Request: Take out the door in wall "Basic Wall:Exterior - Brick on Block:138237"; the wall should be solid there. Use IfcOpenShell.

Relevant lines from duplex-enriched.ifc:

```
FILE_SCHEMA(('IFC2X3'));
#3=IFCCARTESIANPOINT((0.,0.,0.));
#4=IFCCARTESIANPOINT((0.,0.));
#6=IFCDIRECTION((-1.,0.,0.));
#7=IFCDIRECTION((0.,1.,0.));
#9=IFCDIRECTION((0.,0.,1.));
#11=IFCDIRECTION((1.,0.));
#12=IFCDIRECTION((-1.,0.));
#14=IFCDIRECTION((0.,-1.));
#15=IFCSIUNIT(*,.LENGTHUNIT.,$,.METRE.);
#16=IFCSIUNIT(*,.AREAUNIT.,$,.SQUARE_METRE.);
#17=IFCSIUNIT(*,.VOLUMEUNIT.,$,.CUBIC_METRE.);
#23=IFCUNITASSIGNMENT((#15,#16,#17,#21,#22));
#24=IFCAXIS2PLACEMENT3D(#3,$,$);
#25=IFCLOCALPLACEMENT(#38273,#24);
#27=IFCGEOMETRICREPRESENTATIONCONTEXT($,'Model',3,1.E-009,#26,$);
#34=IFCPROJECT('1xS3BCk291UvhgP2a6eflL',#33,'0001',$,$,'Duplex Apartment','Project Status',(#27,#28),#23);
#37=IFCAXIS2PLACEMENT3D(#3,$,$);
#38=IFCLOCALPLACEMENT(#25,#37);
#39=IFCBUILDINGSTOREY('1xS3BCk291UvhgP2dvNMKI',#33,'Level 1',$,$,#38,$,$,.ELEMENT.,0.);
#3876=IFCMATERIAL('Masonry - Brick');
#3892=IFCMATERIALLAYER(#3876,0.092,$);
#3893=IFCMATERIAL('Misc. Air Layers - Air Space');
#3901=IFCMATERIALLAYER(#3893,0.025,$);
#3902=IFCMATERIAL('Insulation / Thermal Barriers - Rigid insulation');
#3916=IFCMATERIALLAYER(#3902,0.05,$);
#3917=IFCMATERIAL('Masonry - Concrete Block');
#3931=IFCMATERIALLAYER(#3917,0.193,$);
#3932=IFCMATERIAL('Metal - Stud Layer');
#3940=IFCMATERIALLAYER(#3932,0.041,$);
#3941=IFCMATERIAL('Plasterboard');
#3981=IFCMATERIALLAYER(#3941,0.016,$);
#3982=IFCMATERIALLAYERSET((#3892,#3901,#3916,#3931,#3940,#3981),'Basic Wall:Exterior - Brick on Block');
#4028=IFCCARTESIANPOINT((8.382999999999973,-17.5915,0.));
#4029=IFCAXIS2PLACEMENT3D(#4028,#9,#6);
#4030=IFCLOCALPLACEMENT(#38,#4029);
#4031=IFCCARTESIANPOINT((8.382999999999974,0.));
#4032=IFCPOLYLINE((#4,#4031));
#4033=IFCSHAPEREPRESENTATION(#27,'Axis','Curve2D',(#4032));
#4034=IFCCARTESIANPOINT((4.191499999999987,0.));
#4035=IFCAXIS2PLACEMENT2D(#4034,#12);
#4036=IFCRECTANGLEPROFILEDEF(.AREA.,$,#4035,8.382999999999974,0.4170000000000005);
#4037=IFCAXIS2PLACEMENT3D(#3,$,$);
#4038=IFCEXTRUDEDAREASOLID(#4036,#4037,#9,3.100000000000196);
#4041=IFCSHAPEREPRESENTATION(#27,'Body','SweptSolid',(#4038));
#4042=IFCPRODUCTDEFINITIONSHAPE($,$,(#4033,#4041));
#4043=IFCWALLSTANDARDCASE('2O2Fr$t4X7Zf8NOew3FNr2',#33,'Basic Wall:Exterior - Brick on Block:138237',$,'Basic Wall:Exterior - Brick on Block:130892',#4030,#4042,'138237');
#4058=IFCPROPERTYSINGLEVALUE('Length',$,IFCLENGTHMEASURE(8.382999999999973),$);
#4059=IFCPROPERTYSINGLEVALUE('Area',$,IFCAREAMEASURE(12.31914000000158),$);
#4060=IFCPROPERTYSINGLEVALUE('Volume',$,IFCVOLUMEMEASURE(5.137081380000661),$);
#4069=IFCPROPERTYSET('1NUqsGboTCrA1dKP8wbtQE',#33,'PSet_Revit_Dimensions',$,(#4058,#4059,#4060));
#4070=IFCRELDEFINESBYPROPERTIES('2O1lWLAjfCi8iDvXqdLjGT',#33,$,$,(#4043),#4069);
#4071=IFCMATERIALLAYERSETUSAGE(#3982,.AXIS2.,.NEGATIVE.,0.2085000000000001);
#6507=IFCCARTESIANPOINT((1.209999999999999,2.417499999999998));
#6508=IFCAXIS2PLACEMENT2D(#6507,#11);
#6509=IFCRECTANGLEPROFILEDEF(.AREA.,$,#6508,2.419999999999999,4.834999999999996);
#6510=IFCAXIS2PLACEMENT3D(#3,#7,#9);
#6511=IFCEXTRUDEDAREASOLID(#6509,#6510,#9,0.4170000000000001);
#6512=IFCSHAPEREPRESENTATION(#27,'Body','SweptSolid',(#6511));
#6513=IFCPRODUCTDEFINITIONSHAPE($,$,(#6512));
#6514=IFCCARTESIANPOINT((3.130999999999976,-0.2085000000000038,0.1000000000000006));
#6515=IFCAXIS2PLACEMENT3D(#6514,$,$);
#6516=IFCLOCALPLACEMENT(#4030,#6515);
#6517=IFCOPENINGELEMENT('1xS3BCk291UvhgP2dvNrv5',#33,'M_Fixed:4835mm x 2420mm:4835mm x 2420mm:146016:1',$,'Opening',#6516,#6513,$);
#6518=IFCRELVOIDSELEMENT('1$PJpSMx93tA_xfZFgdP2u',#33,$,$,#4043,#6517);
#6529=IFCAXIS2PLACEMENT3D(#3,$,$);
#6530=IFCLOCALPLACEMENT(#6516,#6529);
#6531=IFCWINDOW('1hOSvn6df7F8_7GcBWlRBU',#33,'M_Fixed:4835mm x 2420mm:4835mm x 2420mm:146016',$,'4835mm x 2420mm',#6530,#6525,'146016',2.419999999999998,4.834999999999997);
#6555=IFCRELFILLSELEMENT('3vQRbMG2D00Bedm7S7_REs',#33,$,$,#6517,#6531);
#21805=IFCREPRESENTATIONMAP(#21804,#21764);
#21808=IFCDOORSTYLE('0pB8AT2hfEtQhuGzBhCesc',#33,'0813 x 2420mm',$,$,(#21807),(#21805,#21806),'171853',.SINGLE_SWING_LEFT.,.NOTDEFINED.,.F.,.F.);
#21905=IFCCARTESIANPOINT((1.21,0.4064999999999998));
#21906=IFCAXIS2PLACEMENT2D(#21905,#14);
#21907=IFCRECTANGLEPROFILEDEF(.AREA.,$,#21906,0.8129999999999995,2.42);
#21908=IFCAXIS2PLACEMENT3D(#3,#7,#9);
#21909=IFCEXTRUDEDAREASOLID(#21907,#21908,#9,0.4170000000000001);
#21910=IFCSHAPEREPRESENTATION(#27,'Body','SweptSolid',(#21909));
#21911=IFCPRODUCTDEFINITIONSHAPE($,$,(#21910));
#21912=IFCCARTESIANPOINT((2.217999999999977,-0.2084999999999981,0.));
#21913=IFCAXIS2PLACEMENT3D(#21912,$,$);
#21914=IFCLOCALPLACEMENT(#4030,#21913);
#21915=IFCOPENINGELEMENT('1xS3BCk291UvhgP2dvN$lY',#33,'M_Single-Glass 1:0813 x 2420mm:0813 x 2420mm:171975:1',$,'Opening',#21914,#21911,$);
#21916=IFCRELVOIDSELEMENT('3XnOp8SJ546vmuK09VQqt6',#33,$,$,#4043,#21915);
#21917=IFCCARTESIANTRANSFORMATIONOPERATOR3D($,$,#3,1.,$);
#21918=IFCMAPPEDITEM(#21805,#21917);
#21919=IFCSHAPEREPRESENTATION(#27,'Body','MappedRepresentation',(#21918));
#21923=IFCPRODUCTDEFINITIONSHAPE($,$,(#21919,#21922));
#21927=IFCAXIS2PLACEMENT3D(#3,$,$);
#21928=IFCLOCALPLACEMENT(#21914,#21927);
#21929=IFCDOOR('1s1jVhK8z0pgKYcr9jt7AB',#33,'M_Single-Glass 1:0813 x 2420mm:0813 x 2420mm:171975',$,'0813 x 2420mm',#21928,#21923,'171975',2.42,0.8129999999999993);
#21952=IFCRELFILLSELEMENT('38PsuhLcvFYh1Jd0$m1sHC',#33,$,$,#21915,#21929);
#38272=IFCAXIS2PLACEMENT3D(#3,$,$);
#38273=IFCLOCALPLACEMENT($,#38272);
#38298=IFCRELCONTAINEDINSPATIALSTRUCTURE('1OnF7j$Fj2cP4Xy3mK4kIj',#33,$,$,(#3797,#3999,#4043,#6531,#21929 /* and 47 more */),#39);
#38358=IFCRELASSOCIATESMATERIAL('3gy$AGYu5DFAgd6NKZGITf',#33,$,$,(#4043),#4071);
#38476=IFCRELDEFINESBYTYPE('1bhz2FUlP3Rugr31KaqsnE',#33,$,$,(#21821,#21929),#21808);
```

```python
import ifcopenshell
import ifcopenshell.api.feature
import ifcopenshell.api.pset
import ifcopenshell.api.root
import ifcopenshell.geom
import ifcopenshell.util.element
import ifcopenshell.util.shape
import ifcopenshell.util.unit

model = ifcopenshell.open("duplex-enriched.ifc")
area_scale = ifcopenshell.util.unit.calculate_unit_scale(model, "AREAUNIT")
volume_scale = ifcopenshell.util.unit.calculate_unit_scale(model, "VOLUMEUNIT")
settings = ifcopenshell.geom.settings()


def volume(element):
    """Net volume in cubic metres, openings subtracted."""
    shape = ifcopenshell.geom.create_shape(settings, element)
    return ifcopenshell.util.shape.get_volume(shape.geometry)


door = model.by_guid("1s1jVhK8z0pgKYcr9jt7AB")
opening = door.FillsVoids[0].RelatingOpeningElement
wall = opening.VoidsElements[0].RelatingBuildingElement
before = volume(wall)

ifcopenshell.api.root.remove_product(model, product=door)
ifcopenshell.api.feature.remove_feature(model, feature=opening)

after = volume(wall)
thickness = 0.417  # wall thickness in metres

# Update the wall's stored quantities.
pset = model.by_id(ifcopenshell.util.element.get_pset(wall, "PSet_Revit_Dimensions", should_inherit=False)["id"])
ifcopenshell.api.pset.edit_pset(model, pset=pset, properties={
    "Area": model.create_entity("IfcAreaMeasure", after / thickness / area_scale),
    "Volume": model.create_entity("IfcVolumeMeasure", after / volume_scale),
})

print(f"wall volume {before:.3f} -> {after:.3f} m3")

model.write("duplex-enriched_rev.ifc")
```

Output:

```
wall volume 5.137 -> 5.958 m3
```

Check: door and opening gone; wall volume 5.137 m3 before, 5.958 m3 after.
